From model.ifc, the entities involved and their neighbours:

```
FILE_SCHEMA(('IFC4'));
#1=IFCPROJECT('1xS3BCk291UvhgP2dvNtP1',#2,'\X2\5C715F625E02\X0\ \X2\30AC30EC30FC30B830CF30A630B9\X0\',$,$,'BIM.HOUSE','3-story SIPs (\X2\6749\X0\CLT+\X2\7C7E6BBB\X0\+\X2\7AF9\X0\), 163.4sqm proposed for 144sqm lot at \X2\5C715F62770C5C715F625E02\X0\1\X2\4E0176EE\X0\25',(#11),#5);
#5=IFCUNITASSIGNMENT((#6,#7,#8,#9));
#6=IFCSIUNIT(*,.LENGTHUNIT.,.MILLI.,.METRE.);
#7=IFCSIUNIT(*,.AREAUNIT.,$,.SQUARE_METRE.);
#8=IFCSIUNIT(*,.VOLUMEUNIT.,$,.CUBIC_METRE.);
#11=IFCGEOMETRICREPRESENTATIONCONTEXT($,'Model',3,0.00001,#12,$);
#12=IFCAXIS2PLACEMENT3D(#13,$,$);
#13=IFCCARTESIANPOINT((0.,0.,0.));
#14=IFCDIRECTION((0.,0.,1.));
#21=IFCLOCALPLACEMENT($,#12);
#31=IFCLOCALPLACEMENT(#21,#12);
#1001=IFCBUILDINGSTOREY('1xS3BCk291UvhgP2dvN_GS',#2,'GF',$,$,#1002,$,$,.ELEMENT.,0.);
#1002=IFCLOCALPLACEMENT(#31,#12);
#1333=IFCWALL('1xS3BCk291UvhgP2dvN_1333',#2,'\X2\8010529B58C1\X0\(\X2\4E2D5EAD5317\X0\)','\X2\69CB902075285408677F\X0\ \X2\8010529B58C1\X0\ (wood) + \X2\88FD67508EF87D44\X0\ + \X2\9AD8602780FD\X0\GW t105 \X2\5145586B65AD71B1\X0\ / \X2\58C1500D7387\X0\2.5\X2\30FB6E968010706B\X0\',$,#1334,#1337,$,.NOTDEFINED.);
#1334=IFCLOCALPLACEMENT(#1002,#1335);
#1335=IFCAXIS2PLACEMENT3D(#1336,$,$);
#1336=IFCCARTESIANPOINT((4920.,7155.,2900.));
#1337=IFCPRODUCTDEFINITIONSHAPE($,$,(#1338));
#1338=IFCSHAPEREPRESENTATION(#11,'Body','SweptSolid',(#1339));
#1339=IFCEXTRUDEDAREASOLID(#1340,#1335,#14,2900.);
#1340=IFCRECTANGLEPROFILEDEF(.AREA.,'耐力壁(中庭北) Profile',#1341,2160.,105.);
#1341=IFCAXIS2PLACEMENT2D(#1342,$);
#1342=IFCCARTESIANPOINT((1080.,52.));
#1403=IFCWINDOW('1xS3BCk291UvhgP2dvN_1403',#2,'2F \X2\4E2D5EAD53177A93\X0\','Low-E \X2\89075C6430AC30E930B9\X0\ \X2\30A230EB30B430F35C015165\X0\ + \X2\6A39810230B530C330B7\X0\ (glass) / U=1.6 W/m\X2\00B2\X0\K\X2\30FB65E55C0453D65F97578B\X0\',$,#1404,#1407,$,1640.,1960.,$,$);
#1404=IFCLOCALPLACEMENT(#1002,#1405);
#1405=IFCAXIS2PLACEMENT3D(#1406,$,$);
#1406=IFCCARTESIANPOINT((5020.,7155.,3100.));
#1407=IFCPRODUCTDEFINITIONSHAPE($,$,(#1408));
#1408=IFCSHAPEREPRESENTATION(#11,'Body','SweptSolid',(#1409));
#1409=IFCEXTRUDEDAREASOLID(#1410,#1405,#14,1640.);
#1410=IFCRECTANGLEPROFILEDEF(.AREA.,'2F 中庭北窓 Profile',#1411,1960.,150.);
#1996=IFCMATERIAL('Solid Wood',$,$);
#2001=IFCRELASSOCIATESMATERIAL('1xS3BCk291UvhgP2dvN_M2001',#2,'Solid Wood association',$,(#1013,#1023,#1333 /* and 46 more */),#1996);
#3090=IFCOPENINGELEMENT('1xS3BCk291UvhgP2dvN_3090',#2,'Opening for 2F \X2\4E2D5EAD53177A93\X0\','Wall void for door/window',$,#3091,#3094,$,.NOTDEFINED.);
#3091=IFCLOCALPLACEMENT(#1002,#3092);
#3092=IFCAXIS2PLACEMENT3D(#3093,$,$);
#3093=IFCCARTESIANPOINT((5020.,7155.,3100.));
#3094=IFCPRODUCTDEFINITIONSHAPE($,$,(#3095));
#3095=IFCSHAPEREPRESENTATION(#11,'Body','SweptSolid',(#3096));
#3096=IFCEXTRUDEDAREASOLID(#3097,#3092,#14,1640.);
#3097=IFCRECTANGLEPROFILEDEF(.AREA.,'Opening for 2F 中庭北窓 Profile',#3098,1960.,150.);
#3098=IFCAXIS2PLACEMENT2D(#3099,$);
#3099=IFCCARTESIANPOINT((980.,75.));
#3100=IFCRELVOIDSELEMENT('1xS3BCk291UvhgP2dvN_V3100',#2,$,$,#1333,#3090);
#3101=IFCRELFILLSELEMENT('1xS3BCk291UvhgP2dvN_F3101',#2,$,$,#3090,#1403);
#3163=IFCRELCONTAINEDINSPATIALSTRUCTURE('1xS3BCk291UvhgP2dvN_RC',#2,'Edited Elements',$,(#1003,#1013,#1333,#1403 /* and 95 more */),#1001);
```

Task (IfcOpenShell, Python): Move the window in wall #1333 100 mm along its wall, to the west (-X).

```python
import ifcopenshell
import ifcopenshell.api.geometry
import ifcopenshell.util.placement

model = ifcopenshell.open("model.ifc")

window = model.by_id(1403)
opening = window.FillsVoids[0].RelatingOpeningElement
wall = opening.VoidsElements[0].RelatingBuildingElement

wall_matrix = ifcopenshell.util.placement.get_local_placement(wall.ObjectPlacement)
shift = wall_matrix[:3, 0] * -100.0
before = ifcopenshell.util.placement.get_local_placement(window.ObjectPlacement)[:3, 3].copy()

# The window is not placed relative to its opening, so move both.
for product in (opening, window):
    matrix = ifcopenshell.util.placement.get_local_placement(product.ObjectPlacement)
    matrix[:3, 3] += shift
    ifcopenshell.api.geometry.edit_object_placement(model, product=product, matrix=matrix, is_si=False)

after = ifcopenshell.util.placement.get_local_placement(window.ObjectPlacement)[:3, 3]
print("window moved by", (after - before).round(3) + 0.0)

model.write("model-out.ifc")
```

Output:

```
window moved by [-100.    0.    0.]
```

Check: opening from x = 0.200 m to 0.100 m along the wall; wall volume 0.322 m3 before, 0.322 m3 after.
